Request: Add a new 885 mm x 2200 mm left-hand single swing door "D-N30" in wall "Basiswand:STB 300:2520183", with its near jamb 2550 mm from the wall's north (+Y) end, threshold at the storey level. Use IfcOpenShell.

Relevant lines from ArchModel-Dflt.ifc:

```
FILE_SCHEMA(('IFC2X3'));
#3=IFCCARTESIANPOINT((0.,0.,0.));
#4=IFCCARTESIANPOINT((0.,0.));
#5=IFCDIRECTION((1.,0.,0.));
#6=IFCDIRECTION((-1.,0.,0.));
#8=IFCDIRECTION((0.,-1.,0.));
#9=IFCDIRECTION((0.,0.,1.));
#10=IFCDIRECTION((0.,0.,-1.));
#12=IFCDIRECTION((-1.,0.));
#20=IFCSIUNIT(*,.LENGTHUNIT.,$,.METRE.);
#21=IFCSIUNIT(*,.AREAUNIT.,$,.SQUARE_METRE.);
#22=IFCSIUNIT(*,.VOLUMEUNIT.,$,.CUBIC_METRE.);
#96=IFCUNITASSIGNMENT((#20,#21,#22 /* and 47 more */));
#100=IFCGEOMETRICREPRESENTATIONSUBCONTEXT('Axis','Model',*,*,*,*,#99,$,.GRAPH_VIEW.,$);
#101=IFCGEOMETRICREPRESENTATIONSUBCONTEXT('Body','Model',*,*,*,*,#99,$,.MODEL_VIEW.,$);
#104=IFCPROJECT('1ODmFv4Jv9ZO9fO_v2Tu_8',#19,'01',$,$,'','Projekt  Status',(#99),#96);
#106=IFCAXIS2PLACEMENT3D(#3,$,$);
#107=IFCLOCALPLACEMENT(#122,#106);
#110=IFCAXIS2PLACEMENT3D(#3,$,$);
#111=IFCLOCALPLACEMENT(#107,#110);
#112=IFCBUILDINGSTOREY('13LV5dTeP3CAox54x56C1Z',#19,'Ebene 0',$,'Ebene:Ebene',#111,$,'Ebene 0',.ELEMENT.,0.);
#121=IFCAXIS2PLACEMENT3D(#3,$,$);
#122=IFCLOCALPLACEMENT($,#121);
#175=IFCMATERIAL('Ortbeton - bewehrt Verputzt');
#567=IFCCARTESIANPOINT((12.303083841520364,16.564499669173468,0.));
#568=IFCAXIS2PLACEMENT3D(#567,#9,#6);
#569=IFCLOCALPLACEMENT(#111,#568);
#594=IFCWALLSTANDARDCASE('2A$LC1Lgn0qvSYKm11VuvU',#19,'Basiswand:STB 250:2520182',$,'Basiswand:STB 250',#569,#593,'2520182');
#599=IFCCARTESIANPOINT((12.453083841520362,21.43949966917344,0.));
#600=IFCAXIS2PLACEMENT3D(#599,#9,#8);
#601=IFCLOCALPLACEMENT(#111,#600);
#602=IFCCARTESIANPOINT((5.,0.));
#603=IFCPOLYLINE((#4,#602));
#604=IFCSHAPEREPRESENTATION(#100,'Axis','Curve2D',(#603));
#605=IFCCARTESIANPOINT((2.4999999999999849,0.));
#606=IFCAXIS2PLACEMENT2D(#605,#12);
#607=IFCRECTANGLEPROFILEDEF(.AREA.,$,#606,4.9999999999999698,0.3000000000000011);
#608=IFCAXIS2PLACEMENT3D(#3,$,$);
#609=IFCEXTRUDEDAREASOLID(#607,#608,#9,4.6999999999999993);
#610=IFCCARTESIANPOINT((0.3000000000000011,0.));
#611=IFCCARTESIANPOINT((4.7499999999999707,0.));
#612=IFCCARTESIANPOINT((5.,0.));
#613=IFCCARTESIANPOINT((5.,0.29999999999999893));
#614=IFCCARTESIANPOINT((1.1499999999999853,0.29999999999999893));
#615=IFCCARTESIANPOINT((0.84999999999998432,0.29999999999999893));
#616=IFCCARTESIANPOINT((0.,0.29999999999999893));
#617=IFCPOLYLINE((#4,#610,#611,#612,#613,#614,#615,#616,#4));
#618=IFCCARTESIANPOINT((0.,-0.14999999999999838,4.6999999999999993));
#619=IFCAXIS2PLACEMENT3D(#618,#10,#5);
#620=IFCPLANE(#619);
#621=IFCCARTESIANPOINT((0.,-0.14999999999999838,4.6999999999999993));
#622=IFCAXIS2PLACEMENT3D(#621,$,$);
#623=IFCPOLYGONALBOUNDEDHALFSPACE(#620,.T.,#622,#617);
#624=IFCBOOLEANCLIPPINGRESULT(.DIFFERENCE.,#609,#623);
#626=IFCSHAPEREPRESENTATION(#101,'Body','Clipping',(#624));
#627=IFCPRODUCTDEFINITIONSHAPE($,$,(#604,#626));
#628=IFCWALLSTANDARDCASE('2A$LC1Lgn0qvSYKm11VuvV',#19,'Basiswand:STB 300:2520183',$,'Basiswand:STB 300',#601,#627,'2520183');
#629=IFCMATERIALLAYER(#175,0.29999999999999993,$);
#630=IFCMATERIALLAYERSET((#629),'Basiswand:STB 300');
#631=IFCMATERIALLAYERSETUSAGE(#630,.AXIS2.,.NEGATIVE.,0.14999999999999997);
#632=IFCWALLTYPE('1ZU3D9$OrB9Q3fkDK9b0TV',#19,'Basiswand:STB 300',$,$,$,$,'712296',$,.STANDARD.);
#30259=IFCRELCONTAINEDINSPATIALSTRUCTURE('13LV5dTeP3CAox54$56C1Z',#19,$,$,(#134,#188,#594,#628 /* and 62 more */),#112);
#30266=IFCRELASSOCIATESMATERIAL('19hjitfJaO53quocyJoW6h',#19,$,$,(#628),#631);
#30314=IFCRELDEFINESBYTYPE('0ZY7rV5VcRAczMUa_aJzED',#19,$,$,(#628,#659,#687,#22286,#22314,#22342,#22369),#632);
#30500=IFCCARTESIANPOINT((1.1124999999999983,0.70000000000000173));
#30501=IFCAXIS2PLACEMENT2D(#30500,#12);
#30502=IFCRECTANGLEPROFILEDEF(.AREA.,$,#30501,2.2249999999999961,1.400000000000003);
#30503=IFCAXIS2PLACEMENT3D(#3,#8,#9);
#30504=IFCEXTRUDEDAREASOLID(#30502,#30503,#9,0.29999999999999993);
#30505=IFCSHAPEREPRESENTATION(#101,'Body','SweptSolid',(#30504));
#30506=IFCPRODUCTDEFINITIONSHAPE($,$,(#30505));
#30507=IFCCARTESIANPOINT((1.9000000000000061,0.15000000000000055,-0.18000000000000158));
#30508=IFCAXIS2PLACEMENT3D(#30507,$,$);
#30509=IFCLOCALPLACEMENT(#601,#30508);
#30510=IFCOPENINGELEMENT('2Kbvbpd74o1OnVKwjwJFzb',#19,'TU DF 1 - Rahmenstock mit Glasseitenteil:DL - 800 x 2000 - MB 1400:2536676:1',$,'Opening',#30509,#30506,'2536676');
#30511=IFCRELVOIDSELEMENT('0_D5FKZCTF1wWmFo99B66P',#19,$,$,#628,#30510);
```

```python
import numpy as np
import ifcopenshell
import ifcopenshell.api.feature
import ifcopenshell.api.geometry
import ifcopenshell.api.root
import ifcopenshell.api.spatial
import ifcopenshell.api.type
import ifcopenshell.geom
import ifcopenshell.util.element
import ifcopenshell.util.placement
import ifcopenshell.util.representation
import ifcopenshell.util.shape
import ifcopenshell.util.unit

model = ifcopenshell.open("ArchModel-Dflt.ifc")
unit_scale = ifcopenshell.util.unit.calculate_unit_scale(model)
settings = ifcopenshell.geom.settings()


def volume(element):
    """Net volume in cubic metres, openings subtracted."""
    shape = ifcopenshell.geom.create_shape(settings, element)
    return ifcopenshell.util.shape.get_volume(shape.geometry)


wall = model.by_guid("2A$LC1Lgn0qvSYKm11VuvV")
storey = ifcopenshell.util.element.get_container(wall, ifc_class="IfcBuildingStorey")
context = ifcopenshell.util.representation.get_context(model, "Model", "Body", "MODEL_VIEW")
before = volume(wall)

width, height, from_end, sill = 0.885, 2.2, 2.55, 0.0  # metres

# The wall runs along its own X axis, and the end named is its -X end.
wall_shape = ifcopenshell.geom.create_shape(settings, wall)
x, y, z = ifcopenshell.util.shape.get_vertices(wall_shape.geometry).T
start = x.min() + from_end
face, thickness = float(y.min()), float(y.max() - y.min())
wall_matrix = ifcopenshell.util.placement.get_local_placement(wall.ObjectPlacement)
level = ifcopenshell.util.placement.get_local_placement(storey.ObjectPlacement)[2, 3]


def in_wall(x, y):
    """Placement at x, y metres in the wall's axes, at sill height."""
    matrix = wall_matrix.copy()
    matrix[:, 3] = wall_matrix @ np.array([x / unit_scale, y / unit_scale, 0.0, 1.0])
    matrix[2, 3] = level + sill / unit_scale
    return matrix


# Opening: a box that overshoots both wall faces by 50 mm.
opening = ifcopenshell.api.root.create_entity(model, ifc_class="IfcOpeningElement")
box = ifcopenshell.api.geometry.add_wall_representation(
    model, context=context, length=width, height=height, thickness=thickness + 0.1
)
ifcopenshell.api.geometry.assign_representation(model, product=opening, representation=box)
ifcopenshell.api.geometry.edit_object_placement(model, product=opening, matrix=in_wall(start, face - 0.05), is_si=False)
ifcopenshell.api.feature.add_feature(model, feature=opening, element=wall)

door = ifcopenshell.api.root.create_entity(model, ifc_class="IfcDoor", name="D-N30")
door.OverallWidth, door.OverallHeight = width / unit_scale, height / unit_scale
body = ifcopenshell.api.geometry.add_door_representation(
    model,
    context=context,
    overall_width=door.OverallWidth,
    overall_height=door.OverallHeight,
    operation_type="SINGLE_SWING_LEFT",
    lining_properties={"LiningDepth": thickness / unit_scale, "ThresholdDepth": thickness / unit_scale},
)
ifcopenshell.api.geometry.assign_representation(model, product=door, representation=body)
ifcopenshell.api.spatial.assign_container(model, products=[door], relating_structure=storey)
fills = ifcopenshell.api.feature.add_filling(model, opening=opening, element=door)
fills.OwnerHistory = door.OwnerHistory  # required in IFC2X3

# IFC2X3 keeps the operation on the door style.
style = ifcopenshell.api.root.create_entity(model, ifc_class="IfcDoorStyle", name="D-N30")
style.OperationType, style.ConstructionType = "SINGLE_SWING_LEFT", "NOTDEFINED"
style.ParameterTakesPrecedence = style.Sizeable = False
ifcopenshell.api.type.assign_type(model, related_objects=[door], relating_type=style)

# The lining spans the wall, so the door starts at the wall face.
ifcopenshell.api.geometry.edit_object_placement(model, product=door, matrix=in_wall(start, face), is_si=False)

after = volume(wall)

print(f"wall volume {before:.3f} -> {after:.3f} m3")

model.write("ArchModel-Dflt_rev.ifc")
```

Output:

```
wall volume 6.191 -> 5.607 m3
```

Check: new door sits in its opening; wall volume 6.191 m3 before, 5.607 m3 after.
